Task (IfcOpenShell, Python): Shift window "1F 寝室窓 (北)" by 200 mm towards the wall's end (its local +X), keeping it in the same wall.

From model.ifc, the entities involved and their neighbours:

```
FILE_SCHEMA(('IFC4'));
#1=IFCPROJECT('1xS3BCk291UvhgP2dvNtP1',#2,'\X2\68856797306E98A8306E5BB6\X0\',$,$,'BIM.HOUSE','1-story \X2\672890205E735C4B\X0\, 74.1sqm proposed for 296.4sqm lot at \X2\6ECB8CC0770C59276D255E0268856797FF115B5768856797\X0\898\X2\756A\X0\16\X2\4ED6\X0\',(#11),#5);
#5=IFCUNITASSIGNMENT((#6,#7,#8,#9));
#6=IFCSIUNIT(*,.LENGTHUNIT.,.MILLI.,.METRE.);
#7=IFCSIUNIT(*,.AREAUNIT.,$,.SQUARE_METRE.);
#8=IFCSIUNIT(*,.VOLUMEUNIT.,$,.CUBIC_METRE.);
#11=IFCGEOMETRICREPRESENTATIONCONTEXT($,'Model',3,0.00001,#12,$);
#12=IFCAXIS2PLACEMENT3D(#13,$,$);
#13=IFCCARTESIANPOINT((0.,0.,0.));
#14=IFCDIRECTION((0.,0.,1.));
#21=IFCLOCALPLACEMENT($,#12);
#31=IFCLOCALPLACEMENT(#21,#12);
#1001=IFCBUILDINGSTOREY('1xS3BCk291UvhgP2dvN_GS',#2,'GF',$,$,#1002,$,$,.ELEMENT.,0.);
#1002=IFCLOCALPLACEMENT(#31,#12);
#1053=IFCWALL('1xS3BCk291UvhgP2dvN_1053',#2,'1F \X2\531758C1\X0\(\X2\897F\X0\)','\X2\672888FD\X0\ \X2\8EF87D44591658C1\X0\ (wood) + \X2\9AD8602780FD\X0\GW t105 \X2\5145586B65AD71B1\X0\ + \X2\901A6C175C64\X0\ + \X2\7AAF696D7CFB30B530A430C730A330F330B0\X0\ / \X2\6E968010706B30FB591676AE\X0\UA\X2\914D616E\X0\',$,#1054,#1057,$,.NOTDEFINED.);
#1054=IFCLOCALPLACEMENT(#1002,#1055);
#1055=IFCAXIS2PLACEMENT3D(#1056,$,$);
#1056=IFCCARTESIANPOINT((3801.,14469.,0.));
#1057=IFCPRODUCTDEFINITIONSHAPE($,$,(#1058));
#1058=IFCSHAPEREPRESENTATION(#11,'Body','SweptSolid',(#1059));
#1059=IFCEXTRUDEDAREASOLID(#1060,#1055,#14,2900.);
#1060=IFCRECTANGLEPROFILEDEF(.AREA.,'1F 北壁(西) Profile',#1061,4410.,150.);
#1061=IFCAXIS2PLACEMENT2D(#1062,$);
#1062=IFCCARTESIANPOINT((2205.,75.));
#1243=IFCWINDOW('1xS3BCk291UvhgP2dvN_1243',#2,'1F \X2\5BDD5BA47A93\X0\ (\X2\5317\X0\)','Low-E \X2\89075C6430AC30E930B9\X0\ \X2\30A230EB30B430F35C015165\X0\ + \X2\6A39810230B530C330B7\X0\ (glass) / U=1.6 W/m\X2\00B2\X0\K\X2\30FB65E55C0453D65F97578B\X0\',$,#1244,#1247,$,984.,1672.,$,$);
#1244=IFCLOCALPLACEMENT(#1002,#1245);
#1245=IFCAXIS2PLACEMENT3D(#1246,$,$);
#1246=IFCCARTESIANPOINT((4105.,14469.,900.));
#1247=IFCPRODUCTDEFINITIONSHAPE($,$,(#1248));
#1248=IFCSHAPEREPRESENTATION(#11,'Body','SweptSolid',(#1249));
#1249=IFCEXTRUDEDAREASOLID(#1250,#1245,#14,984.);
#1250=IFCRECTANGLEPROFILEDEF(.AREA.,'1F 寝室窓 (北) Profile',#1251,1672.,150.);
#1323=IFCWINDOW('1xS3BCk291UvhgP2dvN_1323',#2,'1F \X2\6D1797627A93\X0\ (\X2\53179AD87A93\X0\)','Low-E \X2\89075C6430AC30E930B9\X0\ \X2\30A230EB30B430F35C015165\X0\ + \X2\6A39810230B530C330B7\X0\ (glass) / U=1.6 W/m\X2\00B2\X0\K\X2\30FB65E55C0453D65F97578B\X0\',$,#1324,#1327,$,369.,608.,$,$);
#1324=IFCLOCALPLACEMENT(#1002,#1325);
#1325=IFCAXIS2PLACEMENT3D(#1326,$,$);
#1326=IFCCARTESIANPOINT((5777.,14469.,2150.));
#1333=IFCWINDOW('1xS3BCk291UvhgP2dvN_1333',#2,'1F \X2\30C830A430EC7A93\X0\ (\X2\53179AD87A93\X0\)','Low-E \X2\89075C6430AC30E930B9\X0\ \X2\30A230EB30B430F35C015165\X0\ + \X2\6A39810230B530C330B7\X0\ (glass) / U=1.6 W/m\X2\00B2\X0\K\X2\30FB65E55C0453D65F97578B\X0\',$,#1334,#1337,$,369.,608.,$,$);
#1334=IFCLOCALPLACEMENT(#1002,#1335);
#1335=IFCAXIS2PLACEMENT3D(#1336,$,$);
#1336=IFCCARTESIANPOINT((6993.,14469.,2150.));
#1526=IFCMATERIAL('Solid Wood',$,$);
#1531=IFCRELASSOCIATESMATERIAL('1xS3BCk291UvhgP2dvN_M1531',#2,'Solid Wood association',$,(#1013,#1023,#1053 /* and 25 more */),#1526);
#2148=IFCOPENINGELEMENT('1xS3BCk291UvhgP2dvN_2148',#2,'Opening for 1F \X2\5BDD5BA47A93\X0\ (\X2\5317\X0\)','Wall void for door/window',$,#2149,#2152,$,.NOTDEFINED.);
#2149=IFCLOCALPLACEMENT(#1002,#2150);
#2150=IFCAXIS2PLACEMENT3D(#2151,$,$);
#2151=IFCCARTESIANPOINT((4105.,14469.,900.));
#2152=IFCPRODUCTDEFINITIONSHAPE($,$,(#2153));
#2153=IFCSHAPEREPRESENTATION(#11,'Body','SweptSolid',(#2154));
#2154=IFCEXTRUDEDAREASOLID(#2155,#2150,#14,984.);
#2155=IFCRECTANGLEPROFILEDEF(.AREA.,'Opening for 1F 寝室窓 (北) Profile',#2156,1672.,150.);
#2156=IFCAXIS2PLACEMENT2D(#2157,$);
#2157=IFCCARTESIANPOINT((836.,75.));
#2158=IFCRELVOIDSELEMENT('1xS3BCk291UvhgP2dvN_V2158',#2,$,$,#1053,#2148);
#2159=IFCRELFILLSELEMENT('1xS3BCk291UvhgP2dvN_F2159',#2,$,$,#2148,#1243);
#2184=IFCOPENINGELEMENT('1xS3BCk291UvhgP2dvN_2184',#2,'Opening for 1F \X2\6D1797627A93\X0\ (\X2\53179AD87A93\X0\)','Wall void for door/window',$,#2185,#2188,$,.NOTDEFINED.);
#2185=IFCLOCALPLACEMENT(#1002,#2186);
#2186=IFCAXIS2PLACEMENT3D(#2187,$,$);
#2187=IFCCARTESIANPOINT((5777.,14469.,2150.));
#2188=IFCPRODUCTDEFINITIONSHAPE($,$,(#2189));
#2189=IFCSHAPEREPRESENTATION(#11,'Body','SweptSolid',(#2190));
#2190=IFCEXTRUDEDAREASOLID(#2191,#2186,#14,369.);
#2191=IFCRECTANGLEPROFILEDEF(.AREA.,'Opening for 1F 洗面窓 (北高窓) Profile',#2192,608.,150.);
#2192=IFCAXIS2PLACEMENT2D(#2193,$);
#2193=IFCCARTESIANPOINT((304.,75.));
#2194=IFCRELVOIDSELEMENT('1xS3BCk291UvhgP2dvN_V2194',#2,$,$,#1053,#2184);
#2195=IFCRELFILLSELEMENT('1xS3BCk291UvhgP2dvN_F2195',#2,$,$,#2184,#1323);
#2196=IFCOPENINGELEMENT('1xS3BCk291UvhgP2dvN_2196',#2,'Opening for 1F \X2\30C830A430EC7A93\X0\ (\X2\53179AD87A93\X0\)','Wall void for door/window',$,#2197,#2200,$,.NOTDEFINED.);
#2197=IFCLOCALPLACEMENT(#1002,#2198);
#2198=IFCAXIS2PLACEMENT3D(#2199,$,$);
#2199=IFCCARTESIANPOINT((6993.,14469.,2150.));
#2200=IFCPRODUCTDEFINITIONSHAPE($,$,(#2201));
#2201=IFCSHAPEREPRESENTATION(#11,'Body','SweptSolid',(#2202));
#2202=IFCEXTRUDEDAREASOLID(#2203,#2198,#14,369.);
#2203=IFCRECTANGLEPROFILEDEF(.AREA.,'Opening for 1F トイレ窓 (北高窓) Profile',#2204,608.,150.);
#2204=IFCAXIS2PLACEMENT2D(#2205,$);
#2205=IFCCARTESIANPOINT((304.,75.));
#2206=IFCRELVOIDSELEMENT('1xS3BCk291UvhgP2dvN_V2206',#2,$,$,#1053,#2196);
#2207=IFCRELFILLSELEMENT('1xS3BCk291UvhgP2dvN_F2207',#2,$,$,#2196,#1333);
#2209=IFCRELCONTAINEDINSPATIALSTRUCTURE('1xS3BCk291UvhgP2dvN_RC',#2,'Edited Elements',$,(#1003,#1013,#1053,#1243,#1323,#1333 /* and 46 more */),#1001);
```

```python
import ifcopenshell
import ifcopenshell.api.geometry
import ifcopenshell.util.placement

model = ifcopenshell.open("model.ifc")

window = model.by_guid("1xS3BCk291UvhgP2dvN_1243")
opening = window.FillsVoids[0].RelatingOpeningElement
wall = opening.VoidsElements[0].RelatingBuildingElement

wall_matrix = ifcopenshell.util.placement.get_local_placement(wall.ObjectPlacement)
shift = wall_matrix[:3, 0] * 200.0
before = ifcopenshell.util.placement.get_local_placement(window.ObjectPlacement)[:3, 3].copy()

# The window is not placed relative to its opening, so move both.
for product in (opening, window):
    matrix = ifcopenshell.util.placement.get_local_placement(product.ObjectPlacement)
    matrix[:3, 3] += shift
    ifcopenshell.api.geometry.edit_object_placement(model, product=product, matrix=matrix, is_si=False)

after = ifcopenshell.util.placement.get_local_placement(window.ObjectPlacement)[:3, 3]
print("window moved by", (after - before).round(3) + 0.0)

model.write("model_edited.ifc")
```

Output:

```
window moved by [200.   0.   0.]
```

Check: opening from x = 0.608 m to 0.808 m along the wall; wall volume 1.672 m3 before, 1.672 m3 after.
